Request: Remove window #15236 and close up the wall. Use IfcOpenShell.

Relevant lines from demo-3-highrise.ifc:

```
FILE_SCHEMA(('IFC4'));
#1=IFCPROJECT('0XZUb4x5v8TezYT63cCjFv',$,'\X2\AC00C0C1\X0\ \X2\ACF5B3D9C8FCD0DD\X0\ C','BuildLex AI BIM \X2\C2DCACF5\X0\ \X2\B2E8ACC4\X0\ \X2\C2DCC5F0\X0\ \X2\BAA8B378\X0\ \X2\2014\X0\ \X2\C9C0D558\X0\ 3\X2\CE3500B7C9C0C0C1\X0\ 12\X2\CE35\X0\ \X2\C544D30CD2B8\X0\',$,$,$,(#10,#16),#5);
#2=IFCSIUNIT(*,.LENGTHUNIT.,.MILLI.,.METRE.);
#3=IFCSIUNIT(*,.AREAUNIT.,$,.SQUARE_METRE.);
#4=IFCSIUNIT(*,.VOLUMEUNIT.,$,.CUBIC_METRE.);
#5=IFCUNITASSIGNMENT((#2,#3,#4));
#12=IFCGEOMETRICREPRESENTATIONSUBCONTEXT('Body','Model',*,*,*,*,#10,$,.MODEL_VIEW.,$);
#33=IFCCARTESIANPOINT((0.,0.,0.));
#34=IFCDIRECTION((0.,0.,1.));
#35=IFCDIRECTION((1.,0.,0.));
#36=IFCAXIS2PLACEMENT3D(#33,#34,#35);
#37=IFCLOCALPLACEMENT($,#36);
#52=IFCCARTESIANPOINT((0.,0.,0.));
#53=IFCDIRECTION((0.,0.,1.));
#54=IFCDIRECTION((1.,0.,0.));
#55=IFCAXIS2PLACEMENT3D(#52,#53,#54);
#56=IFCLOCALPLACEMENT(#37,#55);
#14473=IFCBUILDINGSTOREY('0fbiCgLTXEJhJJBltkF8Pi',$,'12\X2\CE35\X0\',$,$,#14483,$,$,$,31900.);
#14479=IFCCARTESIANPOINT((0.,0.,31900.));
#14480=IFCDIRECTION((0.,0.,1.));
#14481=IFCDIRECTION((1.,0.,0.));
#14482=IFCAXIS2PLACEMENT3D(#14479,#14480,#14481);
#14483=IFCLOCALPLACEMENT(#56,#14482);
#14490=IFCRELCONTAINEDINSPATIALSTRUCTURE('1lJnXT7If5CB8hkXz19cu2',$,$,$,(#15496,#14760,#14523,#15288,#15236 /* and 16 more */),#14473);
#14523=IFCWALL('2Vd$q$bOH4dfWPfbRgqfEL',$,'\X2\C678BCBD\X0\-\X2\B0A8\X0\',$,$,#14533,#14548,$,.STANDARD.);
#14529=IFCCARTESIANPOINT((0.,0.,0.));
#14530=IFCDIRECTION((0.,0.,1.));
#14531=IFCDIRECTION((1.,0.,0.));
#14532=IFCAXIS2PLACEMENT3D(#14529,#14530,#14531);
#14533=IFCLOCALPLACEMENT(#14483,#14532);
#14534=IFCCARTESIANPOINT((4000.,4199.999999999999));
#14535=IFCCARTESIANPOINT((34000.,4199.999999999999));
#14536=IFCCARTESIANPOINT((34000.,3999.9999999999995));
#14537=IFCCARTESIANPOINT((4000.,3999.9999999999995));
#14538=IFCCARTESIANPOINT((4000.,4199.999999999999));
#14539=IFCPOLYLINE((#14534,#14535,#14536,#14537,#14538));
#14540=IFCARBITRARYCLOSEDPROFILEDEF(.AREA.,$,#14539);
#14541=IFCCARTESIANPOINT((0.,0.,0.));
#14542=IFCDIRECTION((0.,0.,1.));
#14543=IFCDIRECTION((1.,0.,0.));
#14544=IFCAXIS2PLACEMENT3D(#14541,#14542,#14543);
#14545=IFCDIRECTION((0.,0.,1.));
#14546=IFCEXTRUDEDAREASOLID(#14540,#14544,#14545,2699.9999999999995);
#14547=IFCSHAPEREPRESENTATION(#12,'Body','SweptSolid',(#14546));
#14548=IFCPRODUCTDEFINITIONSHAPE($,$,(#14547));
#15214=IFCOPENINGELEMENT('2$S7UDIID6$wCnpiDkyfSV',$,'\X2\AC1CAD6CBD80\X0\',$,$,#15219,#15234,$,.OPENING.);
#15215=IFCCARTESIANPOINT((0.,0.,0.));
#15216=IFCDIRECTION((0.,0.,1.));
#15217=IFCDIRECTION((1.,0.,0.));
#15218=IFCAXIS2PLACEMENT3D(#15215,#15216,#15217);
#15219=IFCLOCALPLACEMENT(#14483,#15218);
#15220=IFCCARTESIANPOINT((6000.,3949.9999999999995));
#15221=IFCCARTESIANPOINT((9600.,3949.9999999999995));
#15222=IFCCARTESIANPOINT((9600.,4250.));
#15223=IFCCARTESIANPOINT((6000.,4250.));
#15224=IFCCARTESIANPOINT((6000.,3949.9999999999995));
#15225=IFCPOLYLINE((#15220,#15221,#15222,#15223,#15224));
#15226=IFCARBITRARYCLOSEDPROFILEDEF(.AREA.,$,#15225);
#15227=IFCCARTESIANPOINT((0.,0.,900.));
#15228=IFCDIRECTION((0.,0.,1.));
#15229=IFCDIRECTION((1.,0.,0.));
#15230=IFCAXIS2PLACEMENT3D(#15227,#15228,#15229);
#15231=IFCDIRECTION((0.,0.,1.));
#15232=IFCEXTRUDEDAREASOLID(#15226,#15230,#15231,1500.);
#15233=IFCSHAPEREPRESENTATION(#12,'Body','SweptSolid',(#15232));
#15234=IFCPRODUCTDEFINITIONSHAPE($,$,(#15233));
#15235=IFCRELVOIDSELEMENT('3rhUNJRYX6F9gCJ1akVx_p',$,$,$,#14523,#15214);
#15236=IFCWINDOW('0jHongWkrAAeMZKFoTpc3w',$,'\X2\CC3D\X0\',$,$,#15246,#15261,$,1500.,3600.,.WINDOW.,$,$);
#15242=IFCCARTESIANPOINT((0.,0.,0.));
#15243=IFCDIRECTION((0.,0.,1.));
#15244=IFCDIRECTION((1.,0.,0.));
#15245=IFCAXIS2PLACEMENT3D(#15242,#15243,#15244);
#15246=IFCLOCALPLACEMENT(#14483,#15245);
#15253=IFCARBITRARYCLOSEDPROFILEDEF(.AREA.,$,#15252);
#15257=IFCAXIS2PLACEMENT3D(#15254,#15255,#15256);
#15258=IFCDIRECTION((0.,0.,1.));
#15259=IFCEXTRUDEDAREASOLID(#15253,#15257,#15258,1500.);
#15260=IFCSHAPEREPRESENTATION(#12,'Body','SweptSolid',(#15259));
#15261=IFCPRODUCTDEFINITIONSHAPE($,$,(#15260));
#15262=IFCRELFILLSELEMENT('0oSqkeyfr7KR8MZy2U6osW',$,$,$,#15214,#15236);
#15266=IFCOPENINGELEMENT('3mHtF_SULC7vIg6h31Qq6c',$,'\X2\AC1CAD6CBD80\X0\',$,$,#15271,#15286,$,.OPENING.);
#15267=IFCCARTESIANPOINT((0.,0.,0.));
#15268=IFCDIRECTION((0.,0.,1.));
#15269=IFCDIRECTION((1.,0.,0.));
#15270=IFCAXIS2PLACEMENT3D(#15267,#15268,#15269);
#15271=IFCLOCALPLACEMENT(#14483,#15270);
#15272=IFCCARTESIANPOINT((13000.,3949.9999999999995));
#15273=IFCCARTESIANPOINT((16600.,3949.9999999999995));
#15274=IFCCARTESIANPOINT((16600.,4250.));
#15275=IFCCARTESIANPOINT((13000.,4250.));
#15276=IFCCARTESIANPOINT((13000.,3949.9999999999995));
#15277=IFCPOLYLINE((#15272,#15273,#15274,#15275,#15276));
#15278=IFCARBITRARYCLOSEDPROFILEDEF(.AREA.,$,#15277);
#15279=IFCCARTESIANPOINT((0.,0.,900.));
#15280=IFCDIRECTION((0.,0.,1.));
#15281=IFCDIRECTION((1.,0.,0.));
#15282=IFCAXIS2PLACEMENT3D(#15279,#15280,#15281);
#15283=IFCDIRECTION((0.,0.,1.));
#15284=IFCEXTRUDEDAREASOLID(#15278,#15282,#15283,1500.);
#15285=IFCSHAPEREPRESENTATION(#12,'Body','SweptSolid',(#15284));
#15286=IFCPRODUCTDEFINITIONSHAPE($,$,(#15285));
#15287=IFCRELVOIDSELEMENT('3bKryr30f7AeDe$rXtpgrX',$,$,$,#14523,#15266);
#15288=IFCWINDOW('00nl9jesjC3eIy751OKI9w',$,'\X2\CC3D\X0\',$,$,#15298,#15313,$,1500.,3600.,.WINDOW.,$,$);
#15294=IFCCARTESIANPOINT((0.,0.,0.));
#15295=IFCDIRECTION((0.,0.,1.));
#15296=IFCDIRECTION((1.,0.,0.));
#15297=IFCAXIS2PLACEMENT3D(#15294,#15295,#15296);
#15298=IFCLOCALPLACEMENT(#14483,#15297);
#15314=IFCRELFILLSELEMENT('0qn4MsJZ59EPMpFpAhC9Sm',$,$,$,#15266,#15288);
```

```python
import ifcopenshell
import ifcopenshell.api.feature
import ifcopenshell.api.root
import ifcopenshell.geom
import ifcopenshell.util.shape

model = ifcopenshell.open("demo-3-highrise.ifc")
settings = ifcopenshell.geom.settings()


def volume(element):
    """Net volume in cubic metres, openings subtracted."""
    shape = ifcopenshell.geom.create_shape(settings, element)
    return ifcopenshell.util.shape.get_volume(shape.geometry)


window = model.by_guid("0jHongWkrAAeMZKFoTpc3w")
opening = window.FillsVoids[0].RelatingOpeningElement
wall = opening.VoidsElements[0].RelatingBuildingElement
before = volume(wall)

ifcopenshell.api.root.remove_product(model, product=window)
ifcopenshell.api.feature.remove_feature(model, feature=opening)

after = volume(wall)

print(f"wall volume {before:.3f} -> {after:.3f} m3")

model.write("demo-3-highrise-out.ifc")
```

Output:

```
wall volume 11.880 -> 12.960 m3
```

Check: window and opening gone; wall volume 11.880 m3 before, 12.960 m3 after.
